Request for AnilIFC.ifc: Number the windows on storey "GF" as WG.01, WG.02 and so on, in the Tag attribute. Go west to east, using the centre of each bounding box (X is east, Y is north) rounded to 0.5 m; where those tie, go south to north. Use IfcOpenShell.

First a look at what the model holds.

```python
import ifcopenshell
import ifcopenshell.util.element
import ifcopenshell.util.placement

model = ifcopenshell.open("AnilIFC.ifc")
print(model.schema)
storey = next(s for s in model.by_type("IfcBuildingStorey") if s.Name == "GF")
windows = [e for e in ifcopenshell.util.element.get_decomposition(storey) if e.is_a("IfcWindow")]
for e in sorted(windows, key=lambda e: e.id()):
    origin = ifcopenshell.util.placement.get_local_placement(e.ObjectPlacement)[:3, 3]
    print(e.id(), e.Tag, e.Name, origin.round(2) + 0.0, sep=" | ")
```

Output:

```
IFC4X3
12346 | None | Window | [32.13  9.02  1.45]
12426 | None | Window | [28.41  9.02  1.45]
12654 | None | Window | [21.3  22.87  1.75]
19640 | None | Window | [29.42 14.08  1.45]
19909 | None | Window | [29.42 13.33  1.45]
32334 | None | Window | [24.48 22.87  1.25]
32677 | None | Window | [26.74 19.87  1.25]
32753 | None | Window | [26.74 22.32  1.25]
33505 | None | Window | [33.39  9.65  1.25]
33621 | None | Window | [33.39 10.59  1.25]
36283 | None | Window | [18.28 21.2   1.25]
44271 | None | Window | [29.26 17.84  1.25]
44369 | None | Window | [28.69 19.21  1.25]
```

```python
import ifcopenshell
import ifcopenshell.geom
import ifcopenshell.util.element
import ifcopenshell.util.shape

model = ifcopenshell.open("AnilIFC.ifc")
settings = ifcopenshell.geom.settings()
settings.set("use-world-coords", True)


def centre(element):
    shape = ifcopenshell.geom.create_shape(settings, element)
    return ifcopenshell.util.shape.get_bbox_centroid(shape.geometry)


storey = next(s for s in model.by_type("IfcBuildingStorey") if s.Name == "GF")
windows = [e for e in ifcopenshell.util.element.get_decomposition(storey) if e.is_a("IfcWindow")]

# Insertion points can sit at a corner or the storey origin, so sort by the geometry (in metres).
centres = {e: centre(e) for e in windows}
windows.sort(key=lambda e: (round(centres[e][0] / 0.5), centres[e][1]))

for i, e in enumerate(windows, start=1):
    number = f"WG.{i:02d}"
    e.Tag = number
    print(e.id(), number)

model.write("AnilIFC_updated.ifc")
```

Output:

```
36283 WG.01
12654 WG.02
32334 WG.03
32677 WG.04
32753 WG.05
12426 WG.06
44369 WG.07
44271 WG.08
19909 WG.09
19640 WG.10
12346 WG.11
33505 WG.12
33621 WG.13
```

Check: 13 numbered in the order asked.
